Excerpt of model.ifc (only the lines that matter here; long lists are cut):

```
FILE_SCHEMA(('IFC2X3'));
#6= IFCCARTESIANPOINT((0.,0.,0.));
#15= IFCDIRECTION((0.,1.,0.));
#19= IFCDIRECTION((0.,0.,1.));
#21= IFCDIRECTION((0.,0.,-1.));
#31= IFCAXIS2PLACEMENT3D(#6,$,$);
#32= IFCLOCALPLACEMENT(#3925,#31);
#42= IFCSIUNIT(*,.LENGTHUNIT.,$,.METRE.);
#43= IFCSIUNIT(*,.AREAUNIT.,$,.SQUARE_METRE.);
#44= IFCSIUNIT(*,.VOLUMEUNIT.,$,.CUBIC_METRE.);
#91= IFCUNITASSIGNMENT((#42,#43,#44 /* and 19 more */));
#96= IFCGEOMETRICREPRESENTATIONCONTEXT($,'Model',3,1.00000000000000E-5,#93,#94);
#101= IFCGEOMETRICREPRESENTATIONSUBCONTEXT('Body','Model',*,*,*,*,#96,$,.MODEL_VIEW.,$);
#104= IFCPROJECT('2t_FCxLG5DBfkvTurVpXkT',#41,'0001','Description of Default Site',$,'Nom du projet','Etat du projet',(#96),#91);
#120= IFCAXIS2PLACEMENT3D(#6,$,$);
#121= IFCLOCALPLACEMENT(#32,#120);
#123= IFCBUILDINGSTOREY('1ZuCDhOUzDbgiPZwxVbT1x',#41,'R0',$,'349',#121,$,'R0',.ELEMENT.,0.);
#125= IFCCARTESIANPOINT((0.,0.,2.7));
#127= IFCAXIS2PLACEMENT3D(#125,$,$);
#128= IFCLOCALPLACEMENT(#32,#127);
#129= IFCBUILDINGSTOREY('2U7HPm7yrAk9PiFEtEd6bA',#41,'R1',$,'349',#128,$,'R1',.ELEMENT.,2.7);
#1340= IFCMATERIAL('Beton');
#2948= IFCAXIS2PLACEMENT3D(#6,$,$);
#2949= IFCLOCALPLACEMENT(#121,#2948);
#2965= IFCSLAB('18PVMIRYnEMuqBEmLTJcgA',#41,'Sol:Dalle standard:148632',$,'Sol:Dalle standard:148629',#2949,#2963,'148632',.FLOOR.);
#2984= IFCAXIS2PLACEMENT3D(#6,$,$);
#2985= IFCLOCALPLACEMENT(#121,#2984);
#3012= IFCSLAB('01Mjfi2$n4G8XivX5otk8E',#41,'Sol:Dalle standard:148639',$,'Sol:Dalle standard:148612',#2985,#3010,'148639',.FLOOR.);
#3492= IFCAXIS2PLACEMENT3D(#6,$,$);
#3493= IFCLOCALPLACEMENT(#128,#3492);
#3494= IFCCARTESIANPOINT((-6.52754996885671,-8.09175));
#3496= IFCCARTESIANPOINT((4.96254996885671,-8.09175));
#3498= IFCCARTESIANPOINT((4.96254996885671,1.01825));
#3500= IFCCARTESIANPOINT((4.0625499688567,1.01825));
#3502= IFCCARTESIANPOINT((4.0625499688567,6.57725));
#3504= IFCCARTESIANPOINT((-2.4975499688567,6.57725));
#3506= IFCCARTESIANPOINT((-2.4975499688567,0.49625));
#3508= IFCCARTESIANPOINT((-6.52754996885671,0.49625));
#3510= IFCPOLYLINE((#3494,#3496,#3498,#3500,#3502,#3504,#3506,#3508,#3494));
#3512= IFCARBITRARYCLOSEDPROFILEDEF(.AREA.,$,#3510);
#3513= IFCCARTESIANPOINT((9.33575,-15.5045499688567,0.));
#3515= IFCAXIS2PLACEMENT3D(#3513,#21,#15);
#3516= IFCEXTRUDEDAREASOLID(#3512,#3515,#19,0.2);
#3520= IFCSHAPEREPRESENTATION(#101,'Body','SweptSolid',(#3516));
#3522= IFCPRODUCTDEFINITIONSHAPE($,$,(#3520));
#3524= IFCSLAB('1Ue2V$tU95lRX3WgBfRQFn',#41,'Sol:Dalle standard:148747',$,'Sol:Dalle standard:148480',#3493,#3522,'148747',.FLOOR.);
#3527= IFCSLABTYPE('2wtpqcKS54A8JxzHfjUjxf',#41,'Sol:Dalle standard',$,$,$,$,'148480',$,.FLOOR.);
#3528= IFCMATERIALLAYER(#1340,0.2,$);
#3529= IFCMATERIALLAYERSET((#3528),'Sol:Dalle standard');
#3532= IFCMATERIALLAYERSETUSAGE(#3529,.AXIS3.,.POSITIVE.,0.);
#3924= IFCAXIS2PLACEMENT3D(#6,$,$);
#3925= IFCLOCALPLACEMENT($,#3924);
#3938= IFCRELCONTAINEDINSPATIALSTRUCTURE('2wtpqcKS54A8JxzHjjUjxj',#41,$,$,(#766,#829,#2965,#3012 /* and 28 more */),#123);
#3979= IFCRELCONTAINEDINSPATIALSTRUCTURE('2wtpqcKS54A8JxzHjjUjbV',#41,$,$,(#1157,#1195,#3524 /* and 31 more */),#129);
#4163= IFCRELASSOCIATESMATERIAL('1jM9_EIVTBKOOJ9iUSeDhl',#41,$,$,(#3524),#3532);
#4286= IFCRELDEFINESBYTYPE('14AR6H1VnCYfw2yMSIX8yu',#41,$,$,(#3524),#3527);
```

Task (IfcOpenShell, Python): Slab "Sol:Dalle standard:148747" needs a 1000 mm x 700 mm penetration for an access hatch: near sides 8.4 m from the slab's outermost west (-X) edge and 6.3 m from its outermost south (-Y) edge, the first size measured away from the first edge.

```python
import numpy as np
import ifcopenshell
import ifcopenshell.api.feature
import ifcopenshell.api.geometry
import ifcopenshell.api.root
import ifcopenshell.geom
import ifcopenshell.util.placement
import ifcopenshell.util.representation
import ifcopenshell.util.shape
import ifcopenshell.util.unit

model = ifcopenshell.open("model.ifc")
unit_scale = ifcopenshell.util.unit.calculate_unit_scale(model)
settings = ifcopenshell.geom.settings()


def volume(element):
    """Net volume in cubic metres, openings subtracted."""
    shape = ifcopenshell.geom.create_shape(settings, element)
    return ifcopenshell.util.shape.get_volume(shape.geometry)


slab = model.by_guid("1Ue2V$tU95lRX3WgBfRQFn")
before = volume(slab)

# Extent in the slab's own axes, in metres. The edges named are its -X and -Y sides.
slab_shape = ifcopenshell.geom.create_shape(settings, slab)
vertices = ifcopenshell.util.shape.get_vertices(slab_shape.geometry)
x_min, y_min, bottom = vertices.min(axis=0)
top = vertices[:, 2].max()

opening = ifcopenshell.api.root.create_entity(model, ifc_class="IfcOpeningElement", name="Access hatch opening")
context = ifcopenshell.util.representation.get_context(model, "Model", "Body", "MODEL_VIEW")
width, depth = 1, 0.7
outline = [(0.0, 0.0), (width, 0.0), (width, depth), (0.0, depth), (0.0, 0.0)]
# Overshoot both faces by 50 mm so the cut is clean.
shape = ifcopenshell.api.geometry.add_slab_representation(
    model, context=context, depth=top - bottom + 0.1, polyline=outline
)
ifcopenshell.api.geometry.assign_representation(model, product=opening, representation=shape)

matrix = ifcopenshell.util.placement.get_local_placement(slab.ObjectPlacement)
matrix[:, 3] = matrix @ np.append(np.array([x_min + 8.4, y_min + 6.3, bottom - 0.05]) / unit_scale, 1.0)
ifcopenshell.api.geometry.edit_object_placement(model, product=opening, matrix=matrix, is_si=False)
ifcopenshell.api.feature.add_feature(model, feature=opening, element=slab)

after = volume(slab)

print(f"slab volume {before:.3f} -> {after:.3f} m3")

model.write("model_edited.ifc")
```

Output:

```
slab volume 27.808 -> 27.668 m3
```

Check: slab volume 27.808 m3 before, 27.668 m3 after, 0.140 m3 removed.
